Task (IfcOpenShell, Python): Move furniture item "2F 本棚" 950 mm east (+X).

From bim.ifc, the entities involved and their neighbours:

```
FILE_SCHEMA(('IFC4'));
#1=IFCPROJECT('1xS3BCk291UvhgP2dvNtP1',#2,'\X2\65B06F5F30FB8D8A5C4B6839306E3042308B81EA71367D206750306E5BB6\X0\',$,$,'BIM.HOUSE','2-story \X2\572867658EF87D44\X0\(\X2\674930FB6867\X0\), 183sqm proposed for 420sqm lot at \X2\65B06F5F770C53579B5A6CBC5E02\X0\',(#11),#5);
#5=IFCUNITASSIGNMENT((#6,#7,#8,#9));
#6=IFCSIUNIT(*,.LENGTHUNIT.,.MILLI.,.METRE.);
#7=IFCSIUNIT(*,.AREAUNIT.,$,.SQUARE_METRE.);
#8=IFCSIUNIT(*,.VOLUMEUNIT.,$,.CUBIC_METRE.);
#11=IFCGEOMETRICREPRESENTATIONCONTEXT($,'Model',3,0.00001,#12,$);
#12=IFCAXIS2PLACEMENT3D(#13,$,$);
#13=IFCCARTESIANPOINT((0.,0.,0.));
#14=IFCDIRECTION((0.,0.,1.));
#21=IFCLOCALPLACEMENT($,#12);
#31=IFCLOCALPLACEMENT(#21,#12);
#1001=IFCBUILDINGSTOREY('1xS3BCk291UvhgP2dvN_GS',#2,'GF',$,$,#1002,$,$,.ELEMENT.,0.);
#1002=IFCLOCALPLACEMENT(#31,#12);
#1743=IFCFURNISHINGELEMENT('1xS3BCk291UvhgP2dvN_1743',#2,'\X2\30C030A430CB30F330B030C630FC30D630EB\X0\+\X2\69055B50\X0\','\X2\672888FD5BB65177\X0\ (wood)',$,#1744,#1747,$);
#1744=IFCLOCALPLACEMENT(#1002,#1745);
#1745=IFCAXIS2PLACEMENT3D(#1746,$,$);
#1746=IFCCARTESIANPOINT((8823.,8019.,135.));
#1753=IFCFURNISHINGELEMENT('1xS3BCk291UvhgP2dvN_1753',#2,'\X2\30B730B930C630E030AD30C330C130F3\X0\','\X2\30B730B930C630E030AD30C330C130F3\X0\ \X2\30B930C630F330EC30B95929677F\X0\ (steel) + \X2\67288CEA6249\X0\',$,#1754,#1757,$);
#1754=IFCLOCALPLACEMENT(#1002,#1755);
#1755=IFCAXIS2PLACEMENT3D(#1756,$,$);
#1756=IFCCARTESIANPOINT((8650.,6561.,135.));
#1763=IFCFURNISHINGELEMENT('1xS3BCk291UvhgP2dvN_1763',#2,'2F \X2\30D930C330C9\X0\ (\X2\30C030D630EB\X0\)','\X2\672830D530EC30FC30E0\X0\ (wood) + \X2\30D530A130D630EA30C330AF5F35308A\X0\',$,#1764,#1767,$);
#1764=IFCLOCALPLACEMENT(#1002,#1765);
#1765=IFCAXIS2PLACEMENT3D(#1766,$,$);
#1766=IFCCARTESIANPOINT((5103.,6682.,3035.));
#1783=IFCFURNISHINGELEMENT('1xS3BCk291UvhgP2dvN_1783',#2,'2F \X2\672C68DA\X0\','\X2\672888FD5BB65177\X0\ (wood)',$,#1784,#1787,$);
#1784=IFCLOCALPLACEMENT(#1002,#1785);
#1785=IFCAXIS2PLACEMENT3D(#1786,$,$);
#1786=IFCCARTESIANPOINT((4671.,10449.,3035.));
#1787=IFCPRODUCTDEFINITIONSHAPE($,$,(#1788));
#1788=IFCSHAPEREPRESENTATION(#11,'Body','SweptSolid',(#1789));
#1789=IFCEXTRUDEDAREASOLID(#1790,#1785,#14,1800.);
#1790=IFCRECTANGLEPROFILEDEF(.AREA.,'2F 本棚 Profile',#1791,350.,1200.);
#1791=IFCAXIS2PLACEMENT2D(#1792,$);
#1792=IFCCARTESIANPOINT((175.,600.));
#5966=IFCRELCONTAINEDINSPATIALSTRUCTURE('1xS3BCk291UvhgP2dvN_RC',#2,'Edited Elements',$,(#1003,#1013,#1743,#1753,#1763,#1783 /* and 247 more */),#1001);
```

```python
import ifcopenshell
import ifcopenshell.api.geometry
import ifcopenshell.util.placement
import ifcopenshell.util.unit

model = ifcopenshell.open("bim.ifc")
unit_scale = ifcopenshell.util.unit.calculate_unit_scale(model)

item = model.by_guid("1xS3BCk291UvhgP2dvN_1783")
matrix = ifcopenshell.util.placement.get_local_placement(item.ObjectPlacement)
matrix[0, 3] += 0.95 / unit_scale
ifcopenshell.api.geometry.edit_object_placement(model, product=item, matrix=matrix, is_si=False)

print(ifcopenshell.util.placement.get_local_placement(item.ObjectPlacement).round(3) + 0.0)

model.write("bim_rev.ifc")
```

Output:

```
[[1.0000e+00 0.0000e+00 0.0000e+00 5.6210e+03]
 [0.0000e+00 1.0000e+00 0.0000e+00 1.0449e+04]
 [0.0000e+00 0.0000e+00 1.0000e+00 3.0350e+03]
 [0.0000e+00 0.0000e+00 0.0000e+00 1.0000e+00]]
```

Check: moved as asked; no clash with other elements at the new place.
